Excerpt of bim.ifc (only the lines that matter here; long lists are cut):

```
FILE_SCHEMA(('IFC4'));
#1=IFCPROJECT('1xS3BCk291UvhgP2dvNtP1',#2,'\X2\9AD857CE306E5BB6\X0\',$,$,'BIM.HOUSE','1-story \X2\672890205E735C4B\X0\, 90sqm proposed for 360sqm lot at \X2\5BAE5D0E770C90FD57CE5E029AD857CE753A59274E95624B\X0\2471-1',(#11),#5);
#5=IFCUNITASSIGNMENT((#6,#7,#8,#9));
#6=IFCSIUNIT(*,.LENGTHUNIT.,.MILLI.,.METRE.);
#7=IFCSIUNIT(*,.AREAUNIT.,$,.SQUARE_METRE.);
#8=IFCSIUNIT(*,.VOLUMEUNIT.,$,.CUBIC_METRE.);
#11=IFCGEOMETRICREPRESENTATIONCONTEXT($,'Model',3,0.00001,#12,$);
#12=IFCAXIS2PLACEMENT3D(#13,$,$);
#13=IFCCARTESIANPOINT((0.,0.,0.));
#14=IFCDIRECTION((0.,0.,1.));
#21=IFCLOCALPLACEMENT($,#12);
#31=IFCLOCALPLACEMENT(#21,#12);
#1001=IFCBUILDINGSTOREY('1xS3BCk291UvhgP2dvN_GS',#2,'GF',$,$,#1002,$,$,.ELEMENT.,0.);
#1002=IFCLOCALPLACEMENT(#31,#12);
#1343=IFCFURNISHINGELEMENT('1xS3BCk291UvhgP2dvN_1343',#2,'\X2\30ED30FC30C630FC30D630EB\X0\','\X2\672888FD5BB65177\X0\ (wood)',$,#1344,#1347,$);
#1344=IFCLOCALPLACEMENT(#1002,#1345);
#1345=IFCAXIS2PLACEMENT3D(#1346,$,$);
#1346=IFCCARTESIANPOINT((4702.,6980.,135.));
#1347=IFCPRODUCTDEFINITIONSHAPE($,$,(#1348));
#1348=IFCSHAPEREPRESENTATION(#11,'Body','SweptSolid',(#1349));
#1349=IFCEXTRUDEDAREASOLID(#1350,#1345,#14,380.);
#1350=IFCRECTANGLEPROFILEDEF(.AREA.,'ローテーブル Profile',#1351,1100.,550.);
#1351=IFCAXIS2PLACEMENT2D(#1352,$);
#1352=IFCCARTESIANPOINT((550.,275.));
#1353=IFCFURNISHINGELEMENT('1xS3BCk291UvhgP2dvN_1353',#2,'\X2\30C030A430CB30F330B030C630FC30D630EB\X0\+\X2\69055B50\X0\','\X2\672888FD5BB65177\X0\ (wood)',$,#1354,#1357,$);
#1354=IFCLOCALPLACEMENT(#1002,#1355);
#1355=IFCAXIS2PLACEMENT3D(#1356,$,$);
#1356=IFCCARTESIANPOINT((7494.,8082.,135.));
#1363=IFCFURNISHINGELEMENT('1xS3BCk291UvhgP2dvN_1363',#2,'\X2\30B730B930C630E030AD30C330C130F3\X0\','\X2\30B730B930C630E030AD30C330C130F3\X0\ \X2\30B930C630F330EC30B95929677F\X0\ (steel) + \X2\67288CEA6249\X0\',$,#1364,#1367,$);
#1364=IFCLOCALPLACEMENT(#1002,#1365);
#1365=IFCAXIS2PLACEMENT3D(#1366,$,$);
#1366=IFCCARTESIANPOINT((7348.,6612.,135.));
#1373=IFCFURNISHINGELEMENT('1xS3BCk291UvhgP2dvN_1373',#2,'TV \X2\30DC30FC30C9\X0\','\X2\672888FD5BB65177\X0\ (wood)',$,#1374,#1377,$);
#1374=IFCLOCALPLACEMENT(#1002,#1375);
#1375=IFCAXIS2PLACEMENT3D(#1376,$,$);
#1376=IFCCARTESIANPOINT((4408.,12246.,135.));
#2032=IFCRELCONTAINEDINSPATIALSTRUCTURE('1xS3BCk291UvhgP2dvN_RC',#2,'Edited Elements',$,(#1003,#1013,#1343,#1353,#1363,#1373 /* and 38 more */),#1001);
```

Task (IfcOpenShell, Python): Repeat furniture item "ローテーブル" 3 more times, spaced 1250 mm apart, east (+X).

```python
import numpy as np
import ifcopenshell
import ifcopenshell.api.geometry
import ifcopenshell.api.root
import ifcopenshell.util.element
import ifcopenshell.util.placement
import ifcopenshell.util.unit

model = ifcopenshell.open("bim.ifc")
unit_scale = ifcopenshell.util.unit.calculate_unit_scale(model)


def reuse_history(source, copy):
    """copy_class also copies each property set's owner history, people and application; keep the originals."""
    for rel in copy.IsDefinedBy:
        if rel.is_a("IfcRelDefinesByProperties") and (history := rel.RelatingPropertyDefinition.OwnerHistory):
            rel.RelatingPropertyDefinition.OwnerHistory = source.OwnerHistory
            ifcopenshell.util.element.remove_deep2(model, history)


source = model.by_id(1343)
base = ifcopenshell.util.placement.get_local_placement(source.ObjectPlacement)
step = np.array([1.0, 0.0, 0.0]) * 1.25 / unit_scale

for i in range(1, 4):
    copy = ifcopenshell.api.root.copy_class(model, product=source)
    copy.Representation = ifcopenshell.util.element.copy_deep(
        model, source.Representation, exclude=["IfcGeometricRepresentationContext", "IfcRepresentationMap"]
    )
    reuse_history(source, copy)
    matrix = base.copy()
    matrix[:3, 3] += i * step
    print("added at", matrix[:3, 3].round(3) + 0.0)
    ifcopenshell.api.geometry.edit_object_placement(model, product=copy, matrix=matrix, is_si=False)

model.write("bim-out.ifc")
```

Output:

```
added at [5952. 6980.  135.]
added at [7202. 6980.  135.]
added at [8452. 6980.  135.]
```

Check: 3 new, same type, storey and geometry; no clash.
